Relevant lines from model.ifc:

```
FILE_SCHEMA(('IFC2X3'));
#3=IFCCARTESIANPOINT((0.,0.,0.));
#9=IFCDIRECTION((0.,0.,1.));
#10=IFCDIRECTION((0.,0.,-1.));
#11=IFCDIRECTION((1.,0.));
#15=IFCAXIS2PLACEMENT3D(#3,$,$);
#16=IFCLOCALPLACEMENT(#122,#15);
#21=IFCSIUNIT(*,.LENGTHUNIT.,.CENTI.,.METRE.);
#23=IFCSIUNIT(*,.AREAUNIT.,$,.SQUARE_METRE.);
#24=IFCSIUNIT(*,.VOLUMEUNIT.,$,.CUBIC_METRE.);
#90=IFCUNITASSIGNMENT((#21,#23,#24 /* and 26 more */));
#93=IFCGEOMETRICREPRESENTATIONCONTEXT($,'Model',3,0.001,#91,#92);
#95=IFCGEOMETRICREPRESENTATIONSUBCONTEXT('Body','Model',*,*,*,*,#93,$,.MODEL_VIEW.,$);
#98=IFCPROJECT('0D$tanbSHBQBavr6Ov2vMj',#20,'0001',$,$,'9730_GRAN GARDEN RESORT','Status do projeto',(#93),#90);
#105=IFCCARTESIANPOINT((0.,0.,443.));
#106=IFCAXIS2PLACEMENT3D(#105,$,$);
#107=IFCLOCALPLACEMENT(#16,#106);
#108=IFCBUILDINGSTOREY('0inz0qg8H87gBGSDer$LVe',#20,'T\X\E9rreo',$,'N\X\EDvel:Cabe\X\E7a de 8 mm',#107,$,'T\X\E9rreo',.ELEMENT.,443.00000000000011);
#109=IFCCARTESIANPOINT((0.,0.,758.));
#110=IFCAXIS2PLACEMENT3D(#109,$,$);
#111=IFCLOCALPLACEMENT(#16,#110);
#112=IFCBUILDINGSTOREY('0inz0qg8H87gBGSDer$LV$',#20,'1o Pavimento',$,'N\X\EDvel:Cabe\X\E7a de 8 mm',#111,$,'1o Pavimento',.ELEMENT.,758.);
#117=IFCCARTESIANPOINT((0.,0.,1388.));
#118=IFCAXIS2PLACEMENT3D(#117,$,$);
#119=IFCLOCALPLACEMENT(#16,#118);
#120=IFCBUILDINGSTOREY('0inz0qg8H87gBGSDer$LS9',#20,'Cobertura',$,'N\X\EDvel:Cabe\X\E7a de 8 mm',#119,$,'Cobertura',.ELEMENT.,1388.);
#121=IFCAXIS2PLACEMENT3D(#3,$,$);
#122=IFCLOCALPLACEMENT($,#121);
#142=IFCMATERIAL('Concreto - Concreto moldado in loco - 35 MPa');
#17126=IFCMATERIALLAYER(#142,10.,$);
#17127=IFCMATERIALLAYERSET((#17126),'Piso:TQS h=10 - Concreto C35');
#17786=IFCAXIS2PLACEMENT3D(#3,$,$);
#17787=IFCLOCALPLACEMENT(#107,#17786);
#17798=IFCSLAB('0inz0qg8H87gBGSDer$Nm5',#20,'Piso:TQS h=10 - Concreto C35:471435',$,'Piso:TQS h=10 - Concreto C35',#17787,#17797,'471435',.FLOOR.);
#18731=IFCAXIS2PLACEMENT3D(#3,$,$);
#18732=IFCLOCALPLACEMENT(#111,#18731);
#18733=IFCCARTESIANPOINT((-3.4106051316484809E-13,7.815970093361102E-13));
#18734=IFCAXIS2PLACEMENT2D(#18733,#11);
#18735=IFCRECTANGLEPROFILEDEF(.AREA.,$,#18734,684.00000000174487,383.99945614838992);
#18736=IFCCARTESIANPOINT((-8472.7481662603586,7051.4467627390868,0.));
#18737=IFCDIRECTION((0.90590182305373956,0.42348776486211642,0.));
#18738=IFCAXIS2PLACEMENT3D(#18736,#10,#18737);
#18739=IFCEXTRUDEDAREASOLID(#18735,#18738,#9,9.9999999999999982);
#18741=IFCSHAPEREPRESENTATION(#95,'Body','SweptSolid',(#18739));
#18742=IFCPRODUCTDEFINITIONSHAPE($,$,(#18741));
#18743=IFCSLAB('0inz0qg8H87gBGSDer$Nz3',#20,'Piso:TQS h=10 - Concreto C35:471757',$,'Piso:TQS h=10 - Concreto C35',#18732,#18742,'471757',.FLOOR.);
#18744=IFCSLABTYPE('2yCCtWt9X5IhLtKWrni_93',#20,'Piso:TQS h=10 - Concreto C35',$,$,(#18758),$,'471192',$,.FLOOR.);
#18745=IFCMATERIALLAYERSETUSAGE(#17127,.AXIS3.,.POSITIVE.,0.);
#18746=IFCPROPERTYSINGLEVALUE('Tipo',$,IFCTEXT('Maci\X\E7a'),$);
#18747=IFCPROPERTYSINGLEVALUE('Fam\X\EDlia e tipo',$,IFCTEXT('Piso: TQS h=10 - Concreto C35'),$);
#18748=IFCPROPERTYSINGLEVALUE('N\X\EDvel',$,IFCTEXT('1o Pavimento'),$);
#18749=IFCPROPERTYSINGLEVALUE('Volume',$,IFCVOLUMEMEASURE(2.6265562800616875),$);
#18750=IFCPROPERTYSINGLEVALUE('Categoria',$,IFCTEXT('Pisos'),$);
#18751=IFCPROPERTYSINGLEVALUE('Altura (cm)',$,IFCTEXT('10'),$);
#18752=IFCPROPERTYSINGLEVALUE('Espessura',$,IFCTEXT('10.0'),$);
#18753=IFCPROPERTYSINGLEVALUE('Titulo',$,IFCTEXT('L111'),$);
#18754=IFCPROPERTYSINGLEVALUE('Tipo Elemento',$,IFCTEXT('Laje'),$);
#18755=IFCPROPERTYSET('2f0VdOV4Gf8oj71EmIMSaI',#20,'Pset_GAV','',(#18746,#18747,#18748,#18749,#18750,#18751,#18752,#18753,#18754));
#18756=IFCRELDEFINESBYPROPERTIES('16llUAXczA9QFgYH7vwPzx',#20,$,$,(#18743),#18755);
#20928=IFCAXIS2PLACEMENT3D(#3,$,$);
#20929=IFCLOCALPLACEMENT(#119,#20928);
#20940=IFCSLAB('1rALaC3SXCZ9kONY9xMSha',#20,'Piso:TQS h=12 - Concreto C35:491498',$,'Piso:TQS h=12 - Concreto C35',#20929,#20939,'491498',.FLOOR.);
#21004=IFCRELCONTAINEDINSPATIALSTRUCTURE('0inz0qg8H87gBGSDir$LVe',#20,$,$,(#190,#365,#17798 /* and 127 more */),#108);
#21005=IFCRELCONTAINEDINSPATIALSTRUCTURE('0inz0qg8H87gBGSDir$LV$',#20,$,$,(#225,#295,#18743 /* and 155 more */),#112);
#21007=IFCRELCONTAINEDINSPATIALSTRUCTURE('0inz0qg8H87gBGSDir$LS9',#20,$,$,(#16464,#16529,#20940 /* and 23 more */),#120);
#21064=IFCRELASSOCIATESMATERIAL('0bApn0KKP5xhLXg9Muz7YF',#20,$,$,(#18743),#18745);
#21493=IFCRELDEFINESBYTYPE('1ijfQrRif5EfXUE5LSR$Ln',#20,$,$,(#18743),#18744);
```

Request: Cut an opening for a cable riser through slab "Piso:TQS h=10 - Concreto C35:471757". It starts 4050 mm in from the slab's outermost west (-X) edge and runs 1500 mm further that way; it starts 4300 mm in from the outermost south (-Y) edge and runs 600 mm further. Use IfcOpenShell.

```python
import numpy as np
import ifcopenshell
import ifcopenshell.api.feature
import ifcopenshell.api.geometry
import ifcopenshell.api.pset
import ifcopenshell.api.root
import ifcopenshell.geom
import ifcopenshell.util.element
import ifcopenshell.util.placement
import ifcopenshell.util.representation
import ifcopenshell.util.shape
import ifcopenshell.util.unit

model = ifcopenshell.open("model.ifc")
unit_scale = ifcopenshell.util.unit.calculate_unit_scale(model)
volume_scale = ifcopenshell.util.unit.calculate_unit_scale(model, "VOLUMEUNIT")
settings = ifcopenshell.geom.settings()


def volume(element):
    """Net volume in cubic metres, openings subtracted."""
    shape = ifcopenshell.geom.create_shape(settings, element)
    return ifcopenshell.util.shape.get_volume(shape.geometry)


slab = model.by_guid("0inz0qg8H87gBGSDer$Nz3")
before = volume(slab)

# Extent in the slab's own axes, in metres. The edges named are its -X and -Y sides.
slab_shape = ifcopenshell.geom.create_shape(settings, slab)
vertices = ifcopenshell.util.shape.get_vertices(slab_shape.geometry)
x_min, y_min, bottom = vertices.min(axis=0)
top = vertices[:, 2].max()

opening = ifcopenshell.api.root.create_entity(model, ifc_class="IfcOpeningElement", name="Cable riser opening")
context = ifcopenshell.util.representation.get_context(model, "Model", "Body", "MODEL_VIEW")
width, depth = 1.5, 0.6
outline = [(0.0, 0.0), (width, 0.0), (width, depth), (0.0, depth), (0.0, 0.0)]
# Overshoot both faces by 50 mm so the cut is clean.
shape = ifcopenshell.api.geometry.add_slab_representation(
    model, context=context, depth=top - bottom + 0.1, polyline=outline
)
ifcopenshell.api.geometry.assign_representation(model, product=opening, representation=shape)

matrix = ifcopenshell.util.placement.get_local_placement(slab.ObjectPlacement)
matrix[:, 3] = matrix @ np.append(np.array([x_min + 4.05, y_min + 4.3, bottom - 0.05]) / unit_scale, 1.0)
ifcopenshell.api.geometry.edit_object_placement(model, product=opening, matrix=matrix, is_si=False)
ifcopenshell.api.feature.add_feature(model, feature=opening, element=slab)

after = volume(slab)

# Update the slab's stored quantities.
pset = model.by_id(ifcopenshell.util.element.get_pset(slab, "Pset_GAV", should_inherit=False)["id"])
ifcopenshell.api.pset.edit_pset(model, pset=pset, properties={
    "Volume": model.create_entity("IfcVolumeMeasure", after / volume_scale),
})

print(f"slab volume {before:.3f} -> {after:.3f} m3")

model.write("model_rev.ifc")
```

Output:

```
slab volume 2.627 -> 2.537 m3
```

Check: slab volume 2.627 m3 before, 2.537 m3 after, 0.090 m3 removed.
